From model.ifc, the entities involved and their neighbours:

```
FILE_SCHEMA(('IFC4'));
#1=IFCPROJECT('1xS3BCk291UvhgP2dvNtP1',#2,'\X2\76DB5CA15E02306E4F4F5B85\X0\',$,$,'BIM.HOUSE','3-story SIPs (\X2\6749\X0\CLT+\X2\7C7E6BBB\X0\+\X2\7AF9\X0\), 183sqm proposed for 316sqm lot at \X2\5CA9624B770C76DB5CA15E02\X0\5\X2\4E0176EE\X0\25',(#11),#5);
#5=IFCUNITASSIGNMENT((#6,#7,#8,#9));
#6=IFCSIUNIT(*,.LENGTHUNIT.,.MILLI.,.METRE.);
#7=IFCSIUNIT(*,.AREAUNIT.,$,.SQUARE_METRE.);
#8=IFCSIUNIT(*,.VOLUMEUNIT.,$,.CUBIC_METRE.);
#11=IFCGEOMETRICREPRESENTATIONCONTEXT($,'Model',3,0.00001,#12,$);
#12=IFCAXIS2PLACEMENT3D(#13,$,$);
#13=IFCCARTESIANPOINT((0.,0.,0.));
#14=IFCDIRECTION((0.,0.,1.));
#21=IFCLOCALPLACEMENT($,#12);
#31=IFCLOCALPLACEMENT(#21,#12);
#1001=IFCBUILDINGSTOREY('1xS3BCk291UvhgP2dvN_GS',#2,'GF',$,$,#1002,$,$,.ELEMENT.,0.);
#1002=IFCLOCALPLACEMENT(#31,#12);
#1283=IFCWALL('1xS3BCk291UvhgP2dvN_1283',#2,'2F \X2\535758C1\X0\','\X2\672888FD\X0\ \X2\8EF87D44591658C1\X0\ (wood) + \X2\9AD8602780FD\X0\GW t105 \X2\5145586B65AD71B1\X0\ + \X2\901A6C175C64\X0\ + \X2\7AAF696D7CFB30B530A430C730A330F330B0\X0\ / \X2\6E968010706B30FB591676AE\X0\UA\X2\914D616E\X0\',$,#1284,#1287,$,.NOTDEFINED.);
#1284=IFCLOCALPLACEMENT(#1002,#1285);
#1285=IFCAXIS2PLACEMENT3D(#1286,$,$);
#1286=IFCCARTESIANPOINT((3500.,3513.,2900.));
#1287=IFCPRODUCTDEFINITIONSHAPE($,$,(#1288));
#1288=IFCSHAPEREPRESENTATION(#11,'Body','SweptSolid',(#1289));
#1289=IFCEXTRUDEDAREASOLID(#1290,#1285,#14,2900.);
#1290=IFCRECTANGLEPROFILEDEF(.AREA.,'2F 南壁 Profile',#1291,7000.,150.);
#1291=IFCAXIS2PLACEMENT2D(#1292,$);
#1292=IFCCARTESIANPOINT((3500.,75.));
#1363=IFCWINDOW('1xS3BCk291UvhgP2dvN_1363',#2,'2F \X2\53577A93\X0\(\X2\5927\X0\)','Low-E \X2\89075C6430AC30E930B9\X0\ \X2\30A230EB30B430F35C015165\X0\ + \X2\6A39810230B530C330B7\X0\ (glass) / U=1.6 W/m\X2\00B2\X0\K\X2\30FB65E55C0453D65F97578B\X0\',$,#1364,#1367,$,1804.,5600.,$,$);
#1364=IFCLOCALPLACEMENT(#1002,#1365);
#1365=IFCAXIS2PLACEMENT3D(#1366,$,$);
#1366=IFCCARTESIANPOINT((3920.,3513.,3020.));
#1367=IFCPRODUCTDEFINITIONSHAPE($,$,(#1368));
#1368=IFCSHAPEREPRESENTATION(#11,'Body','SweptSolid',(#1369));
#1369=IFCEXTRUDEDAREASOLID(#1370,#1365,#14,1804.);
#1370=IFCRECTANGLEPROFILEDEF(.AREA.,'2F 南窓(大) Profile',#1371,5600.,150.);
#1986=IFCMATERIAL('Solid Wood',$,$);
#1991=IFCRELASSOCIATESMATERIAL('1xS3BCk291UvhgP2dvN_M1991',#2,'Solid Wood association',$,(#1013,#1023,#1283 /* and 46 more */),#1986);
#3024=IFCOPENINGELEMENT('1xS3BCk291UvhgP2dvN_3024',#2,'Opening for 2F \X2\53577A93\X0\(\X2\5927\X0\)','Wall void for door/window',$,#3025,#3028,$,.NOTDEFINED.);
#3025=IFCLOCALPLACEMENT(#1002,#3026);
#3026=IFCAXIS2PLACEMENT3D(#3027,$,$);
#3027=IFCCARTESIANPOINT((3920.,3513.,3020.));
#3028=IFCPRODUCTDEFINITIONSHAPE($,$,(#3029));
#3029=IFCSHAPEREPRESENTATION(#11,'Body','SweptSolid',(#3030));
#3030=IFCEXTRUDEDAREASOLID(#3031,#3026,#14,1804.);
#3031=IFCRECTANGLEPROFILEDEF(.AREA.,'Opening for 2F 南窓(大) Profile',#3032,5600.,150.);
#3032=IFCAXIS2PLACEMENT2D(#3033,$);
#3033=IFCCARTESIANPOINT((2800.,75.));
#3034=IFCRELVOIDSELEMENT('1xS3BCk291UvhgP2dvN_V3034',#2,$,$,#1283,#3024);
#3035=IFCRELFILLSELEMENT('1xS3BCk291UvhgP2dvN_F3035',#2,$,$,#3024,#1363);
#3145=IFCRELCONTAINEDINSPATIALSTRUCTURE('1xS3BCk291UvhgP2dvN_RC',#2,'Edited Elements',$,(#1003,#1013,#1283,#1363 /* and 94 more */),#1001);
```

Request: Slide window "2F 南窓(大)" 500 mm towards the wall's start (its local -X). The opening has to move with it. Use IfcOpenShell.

```python
import ifcopenshell
import ifcopenshell.api.geometry
import ifcopenshell.util.placement
import ifcopenshell.util.unit

model = ifcopenshell.open("model.ifc")
unit_scale = ifcopenshell.util.unit.calculate_unit_scale(model)

window = model.by_id(1363)
opening = window.FillsVoids[0].RelatingOpeningElement
wall = opening.VoidsElements[0].RelatingBuildingElement

wall_matrix = ifcopenshell.util.placement.get_local_placement(wall.ObjectPlacement)
shift = wall_matrix[:3, 0] * -0.5 / unit_scale
before = ifcopenshell.util.placement.get_local_placement(window.ObjectPlacement)[:3, 3].copy()

# The window is not placed relative to its opening, so move both.
for product in (opening, window):
    matrix = ifcopenshell.util.placement.get_local_placement(product.ObjectPlacement)
    matrix[:3, 3] += shift
    ifcopenshell.api.geometry.edit_object_placement(model, product=product, matrix=matrix, is_si=False)

after = ifcopenshell.util.placement.get_local_placement(window.ObjectPlacement)[:3, 3]
print("window moved by", (after - before).round(3) + 0.0)

model.write("model_rev.ifc")
```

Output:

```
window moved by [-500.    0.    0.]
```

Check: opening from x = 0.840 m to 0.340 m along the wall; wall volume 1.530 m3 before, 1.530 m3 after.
